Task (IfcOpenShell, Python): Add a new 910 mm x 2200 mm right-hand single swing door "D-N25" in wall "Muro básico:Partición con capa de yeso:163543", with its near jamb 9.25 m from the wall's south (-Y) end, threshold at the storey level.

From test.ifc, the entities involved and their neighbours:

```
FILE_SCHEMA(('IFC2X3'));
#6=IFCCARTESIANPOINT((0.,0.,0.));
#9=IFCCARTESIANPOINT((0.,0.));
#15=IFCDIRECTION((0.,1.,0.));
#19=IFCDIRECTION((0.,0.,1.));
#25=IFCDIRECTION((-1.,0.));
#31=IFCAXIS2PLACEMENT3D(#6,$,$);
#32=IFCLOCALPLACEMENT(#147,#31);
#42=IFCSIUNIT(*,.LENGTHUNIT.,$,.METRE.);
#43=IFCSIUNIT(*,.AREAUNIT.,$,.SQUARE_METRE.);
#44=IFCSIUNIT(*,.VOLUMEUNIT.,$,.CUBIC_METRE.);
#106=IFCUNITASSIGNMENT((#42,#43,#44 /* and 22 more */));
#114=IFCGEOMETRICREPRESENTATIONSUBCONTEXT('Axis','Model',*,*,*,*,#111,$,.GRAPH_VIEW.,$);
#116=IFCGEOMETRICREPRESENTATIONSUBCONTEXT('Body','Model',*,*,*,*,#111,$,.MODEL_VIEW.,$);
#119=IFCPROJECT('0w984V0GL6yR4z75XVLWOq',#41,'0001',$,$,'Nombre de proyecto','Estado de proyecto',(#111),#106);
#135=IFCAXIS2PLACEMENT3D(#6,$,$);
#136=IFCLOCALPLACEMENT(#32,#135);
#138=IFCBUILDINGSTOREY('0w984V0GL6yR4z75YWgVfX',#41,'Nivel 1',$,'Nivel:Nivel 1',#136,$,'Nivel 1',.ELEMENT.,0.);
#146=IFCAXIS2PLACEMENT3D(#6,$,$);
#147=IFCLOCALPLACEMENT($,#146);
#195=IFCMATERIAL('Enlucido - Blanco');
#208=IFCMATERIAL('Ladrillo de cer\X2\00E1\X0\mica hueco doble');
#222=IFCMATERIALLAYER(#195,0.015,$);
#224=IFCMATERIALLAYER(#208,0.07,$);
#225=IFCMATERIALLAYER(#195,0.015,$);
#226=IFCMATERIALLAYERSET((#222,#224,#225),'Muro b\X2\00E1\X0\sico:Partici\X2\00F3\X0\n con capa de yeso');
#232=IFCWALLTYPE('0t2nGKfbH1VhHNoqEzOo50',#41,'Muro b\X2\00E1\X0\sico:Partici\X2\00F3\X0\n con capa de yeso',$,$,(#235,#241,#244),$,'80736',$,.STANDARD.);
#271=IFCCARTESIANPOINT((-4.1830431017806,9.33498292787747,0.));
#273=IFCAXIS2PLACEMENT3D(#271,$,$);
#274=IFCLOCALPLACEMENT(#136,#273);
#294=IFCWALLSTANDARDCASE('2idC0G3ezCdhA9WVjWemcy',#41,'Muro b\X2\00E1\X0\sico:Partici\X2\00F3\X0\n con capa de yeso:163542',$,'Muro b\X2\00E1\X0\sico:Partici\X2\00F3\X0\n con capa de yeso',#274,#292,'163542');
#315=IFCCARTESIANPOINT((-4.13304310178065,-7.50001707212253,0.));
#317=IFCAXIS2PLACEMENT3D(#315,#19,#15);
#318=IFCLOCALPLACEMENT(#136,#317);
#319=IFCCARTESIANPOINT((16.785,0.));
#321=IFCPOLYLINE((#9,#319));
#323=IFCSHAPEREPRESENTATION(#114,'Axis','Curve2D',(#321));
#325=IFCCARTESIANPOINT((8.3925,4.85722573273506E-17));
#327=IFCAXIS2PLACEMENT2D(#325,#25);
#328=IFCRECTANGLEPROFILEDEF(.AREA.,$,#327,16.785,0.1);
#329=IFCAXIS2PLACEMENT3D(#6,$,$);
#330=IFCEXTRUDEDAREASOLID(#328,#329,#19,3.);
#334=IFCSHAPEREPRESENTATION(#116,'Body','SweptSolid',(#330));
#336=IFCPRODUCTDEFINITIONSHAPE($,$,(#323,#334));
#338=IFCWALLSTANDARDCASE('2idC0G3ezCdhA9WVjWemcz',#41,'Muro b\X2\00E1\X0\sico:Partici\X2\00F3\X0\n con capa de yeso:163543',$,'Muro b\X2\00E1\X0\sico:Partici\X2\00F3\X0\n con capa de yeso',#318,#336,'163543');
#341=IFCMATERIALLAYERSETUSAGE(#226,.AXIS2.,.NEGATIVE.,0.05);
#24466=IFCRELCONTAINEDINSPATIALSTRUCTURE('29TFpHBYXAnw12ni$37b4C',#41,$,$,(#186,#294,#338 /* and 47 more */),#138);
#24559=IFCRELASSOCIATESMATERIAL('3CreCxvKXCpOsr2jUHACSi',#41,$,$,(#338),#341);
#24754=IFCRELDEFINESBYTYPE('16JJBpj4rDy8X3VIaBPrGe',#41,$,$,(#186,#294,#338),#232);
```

```python
import numpy as np
import ifcopenshell
import ifcopenshell.api.feature
import ifcopenshell.api.geometry
import ifcopenshell.api.root
import ifcopenshell.api.spatial
import ifcopenshell.api.type
import ifcopenshell.geom
import ifcopenshell.util.element
import ifcopenshell.util.placement
import ifcopenshell.util.representation
import ifcopenshell.util.shape
import ifcopenshell.util.unit

model = ifcopenshell.open("test.ifc")
unit_scale = ifcopenshell.util.unit.calculate_unit_scale(model)
settings = ifcopenshell.geom.settings()


def volume(element):
    """Net volume in cubic metres, openings subtracted."""
    shape = ifcopenshell.geom.create_shape(settings, element)
    return ifcopenshell.util.shape.get_volume(shape.geometry)


wall = model.by_id(338)
storey = ifcopenshell.util.element.get_container(wall, ifc_class="IfcBuildingStorey")
context = ifcopenshell.util.representation.get_context(model, "Model", "Body", "MODEL_VIEW")
before = volume(wall)

width, height, from_end, sill = 0.91, 2.2, 9.25, 0.0  # metres

# The wall runs along its own X axis, and the end named is its -X end.
wall_shape = ifcopenshell.geom.create_shape(settings, wall)
x, y, z = ifcopenshell.util.shape.get_vertices(wall_shape.geometry).T
start = x.min() + from_end
face, thickness = float(y.min()), float(y.max() - y.min())
wall_matrix = ifcopenshell.util.placement.get_local_placement(wall.ObjectPlacement)
level = ifcopenshell.util.placement.get_local_placement(storey.ObjectPlacement)[2, 3]


def in_wall(x, y):
    """Placement at x, y metres in the wall's axes, at sill height."""
    matrix = wall_matrix.copy()
    matrix[:, 3] = wall_matrix @ np.array([x / unit_scale, y / unit_scale, 0.0, 1.0])
    matrix[2, 3] = level + sill / unit_scale
    return matrix


# Opening: a box that overshoots both wall faces by 50 mm.
opening = ifcopenshell.api.root.create_entity(model, ifc_class="IfcOpeningElement")
box = ifcopenshell.api.geometry.add_wall_representation(
    model, context=context, length=width, height=height, thickness=thickness + 0.1
)
ifcopenshell.api.geometry.assign_representation(model, product=opening, representation=box)
ifcopenshell.api.geometry.edit_object_placement(model, product=opening, matrix=in_wall(start, face - 0.05), is_si=False)
ifcopenshell.api.feature.add_feature(model, feature=opening, element=wall)

door = ifcopenshell.api.root.create_entity(model, ifc_class="IfcDoor", name="D-N25")
door.OverallWidth, door.OverallHeight = width / unit_scale, height / unit_scale
body = ifcopenshell.api.geometry.add_door_representation(
    model,
    context=context,
    overall_width=door.OverallWidth,
    overall_height=door.OverallHeight,
    operation_type="SINGLE_SWING_RIGHT",
    lining_properties={"LiningDepth": thickness / unit_scale, "ThresholdDepth": thickness / unit_scale},
)
ifcopenshell.api.geometry.assign_representation(model, product=door, representation=body)
ifcopenshell.api.spatial.assign_container(model, products=[door], relating_structure=storey)
fills = ifcopenshell.api.feature.add_filling(model, opening=opening, element=door)
fills.OwnerHistory = door.OwnerHistory  # required in IFC2X3

# IFC2X3 keeps the operation on the door style.
style = ifcopenshell.api.root.create_entity(model, ifc_class="IfcDoorStyle", name="D-N25")
style.OperationType, style.ConstructionType = "SINGLE_SWING_RIGHT", "NOTDEFINED"
style.ParameterTakesPrecedence = style.Sizeable = False
ifcopenshell.api.type.assign_type(model, related_objects=[door], relating_type=style)

# The lining spans the wall, so the door starts at the wall face.
ifcopenshell.api.geometry.edit_object_placement(model, product=door, matrix=in_wall(start, face), is_si=False)

after = volume(wall)

print(f"wall volume {before:.3f} -> {after:.3f} m3")

model.write("test_edited.ifc")
```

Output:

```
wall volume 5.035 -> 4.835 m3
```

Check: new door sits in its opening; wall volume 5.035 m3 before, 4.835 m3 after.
